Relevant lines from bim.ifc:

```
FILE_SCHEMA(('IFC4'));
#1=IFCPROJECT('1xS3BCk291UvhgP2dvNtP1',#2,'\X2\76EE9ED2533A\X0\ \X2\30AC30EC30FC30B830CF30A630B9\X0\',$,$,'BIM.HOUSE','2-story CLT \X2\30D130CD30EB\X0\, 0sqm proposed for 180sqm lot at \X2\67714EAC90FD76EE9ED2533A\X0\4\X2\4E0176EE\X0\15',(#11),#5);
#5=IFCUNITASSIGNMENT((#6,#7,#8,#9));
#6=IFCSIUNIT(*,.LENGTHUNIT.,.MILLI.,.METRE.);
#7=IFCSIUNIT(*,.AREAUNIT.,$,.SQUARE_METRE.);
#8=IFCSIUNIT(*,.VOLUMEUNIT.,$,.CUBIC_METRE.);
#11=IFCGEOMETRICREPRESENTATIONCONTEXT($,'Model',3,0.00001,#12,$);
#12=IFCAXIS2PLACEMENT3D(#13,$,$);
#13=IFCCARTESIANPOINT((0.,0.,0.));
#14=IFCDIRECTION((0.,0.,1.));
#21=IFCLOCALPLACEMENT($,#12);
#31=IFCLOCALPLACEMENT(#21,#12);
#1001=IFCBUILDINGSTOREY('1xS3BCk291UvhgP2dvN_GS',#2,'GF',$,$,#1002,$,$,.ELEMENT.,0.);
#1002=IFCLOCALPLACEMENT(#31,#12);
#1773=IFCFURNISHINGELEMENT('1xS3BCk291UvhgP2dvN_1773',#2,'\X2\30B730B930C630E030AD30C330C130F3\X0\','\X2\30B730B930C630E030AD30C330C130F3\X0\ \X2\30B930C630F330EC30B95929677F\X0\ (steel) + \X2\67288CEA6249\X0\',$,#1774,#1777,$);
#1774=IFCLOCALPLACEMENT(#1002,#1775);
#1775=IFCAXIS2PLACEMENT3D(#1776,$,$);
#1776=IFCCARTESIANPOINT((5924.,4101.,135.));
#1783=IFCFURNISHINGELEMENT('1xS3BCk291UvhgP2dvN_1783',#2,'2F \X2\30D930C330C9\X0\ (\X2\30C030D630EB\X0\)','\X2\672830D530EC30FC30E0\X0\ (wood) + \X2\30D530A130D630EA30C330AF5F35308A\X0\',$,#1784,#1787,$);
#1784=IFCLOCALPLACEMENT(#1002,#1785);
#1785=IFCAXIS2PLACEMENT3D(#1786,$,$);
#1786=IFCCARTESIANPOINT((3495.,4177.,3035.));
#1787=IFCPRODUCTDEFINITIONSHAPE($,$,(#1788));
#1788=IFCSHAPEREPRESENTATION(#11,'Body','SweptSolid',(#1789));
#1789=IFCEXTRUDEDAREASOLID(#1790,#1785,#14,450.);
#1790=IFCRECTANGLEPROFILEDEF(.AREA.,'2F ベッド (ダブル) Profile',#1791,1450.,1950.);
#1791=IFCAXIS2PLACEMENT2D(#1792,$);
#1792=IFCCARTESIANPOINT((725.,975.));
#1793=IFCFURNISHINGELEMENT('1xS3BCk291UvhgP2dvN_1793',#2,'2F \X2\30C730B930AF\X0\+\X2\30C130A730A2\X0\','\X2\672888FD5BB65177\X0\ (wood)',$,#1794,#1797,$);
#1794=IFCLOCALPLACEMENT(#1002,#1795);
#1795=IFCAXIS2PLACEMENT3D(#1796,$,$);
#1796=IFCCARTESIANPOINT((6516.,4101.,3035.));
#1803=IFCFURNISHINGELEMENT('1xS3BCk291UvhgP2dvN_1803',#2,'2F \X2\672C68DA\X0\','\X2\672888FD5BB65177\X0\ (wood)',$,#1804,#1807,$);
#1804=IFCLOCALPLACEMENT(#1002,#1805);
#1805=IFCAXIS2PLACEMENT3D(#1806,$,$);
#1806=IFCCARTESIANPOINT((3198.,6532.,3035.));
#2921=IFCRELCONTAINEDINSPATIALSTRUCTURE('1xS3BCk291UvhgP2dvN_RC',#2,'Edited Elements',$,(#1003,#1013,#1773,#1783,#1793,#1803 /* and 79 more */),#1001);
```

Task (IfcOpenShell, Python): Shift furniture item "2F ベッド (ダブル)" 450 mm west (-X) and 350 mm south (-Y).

```python
import ifcopenshell
import ifcopenshell.api.geometry
import ifcopenshell.util.placement

model = ifcopenshell.open("bim.ifc")

item = model.by_guid("1xS3BCk291UvhgP2dvN_1783")
matrix = ifcopenshell.util.placement.get_local_placement(item.ObjectPlacement)
matrix[0, 3] -= 450.0
matrix[1, 3] -= 350.0
ifcopenshell.api.geometry.edit_object_placement(model, product=item, matrix=matrix, is_si=False)

print(ifcopenshell.util.placement.get_local_placement(item.ObjectPlacement).round(3) + 0.0)

model.write("bim_rev.ifc")
```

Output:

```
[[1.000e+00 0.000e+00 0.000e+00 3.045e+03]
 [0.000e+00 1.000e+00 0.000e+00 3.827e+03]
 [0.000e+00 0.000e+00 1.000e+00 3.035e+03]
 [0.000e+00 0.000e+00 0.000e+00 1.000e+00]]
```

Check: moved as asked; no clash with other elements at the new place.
